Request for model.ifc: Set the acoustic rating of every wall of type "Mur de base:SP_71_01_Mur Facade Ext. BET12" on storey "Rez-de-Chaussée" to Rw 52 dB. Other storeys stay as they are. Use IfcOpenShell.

First a look at what the model holds.

```python
import ifcopenshell
import ifcopenshell.util.element

model = ifcopenshell.open("model.ifc")
print(model.schema)
storey = next(s for s in model.by_type("IfcBuildingStorey") if s.Name == "Rez-de-Chaussée")
walls = [e for e in ifcopenshell.util.element.get_decomposition(storey) if e.is_a("IfcWall")]
seen = {}
for e in walls:
    element_type = ifcopenshell.util.element.get_type(e)
    key = (element_type.Name if element_type != e and element_type else None, ifcopenshell.util.element.get_pset(e, "Pset_WallCommon", "AcousticRating"))
    seen[key] = seen.get(key, 0) + 1
for (name, value), count in sorted(seen.items(), key=str):
    print(count, "x", name, "|", value)
```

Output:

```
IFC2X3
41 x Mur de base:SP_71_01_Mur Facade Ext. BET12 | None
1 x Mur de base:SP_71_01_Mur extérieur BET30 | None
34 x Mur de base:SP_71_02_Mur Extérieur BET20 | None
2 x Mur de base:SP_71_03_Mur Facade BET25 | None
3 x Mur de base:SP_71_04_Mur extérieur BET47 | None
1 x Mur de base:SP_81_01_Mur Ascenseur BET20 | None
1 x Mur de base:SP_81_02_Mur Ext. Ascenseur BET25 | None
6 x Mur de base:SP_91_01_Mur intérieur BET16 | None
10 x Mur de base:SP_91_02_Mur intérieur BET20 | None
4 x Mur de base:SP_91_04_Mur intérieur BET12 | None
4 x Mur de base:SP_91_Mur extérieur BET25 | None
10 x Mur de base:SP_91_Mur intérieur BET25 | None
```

```python
import ifcopenshell
import ifcopenshell.api.pset
import ifcopenshell.util.element

model = ifcopenshell.open("model.ifc")

storey = next(s for s in model.by_type("IfcBuildingStorey") if s.Name == "Rez-de-Chaussée")
walls = [e for e in ifcopenshell.util.element.get_decomposition(storey) if e.is_a("IfcWall")]

count = 0
for e in walls:
    element_type = ifcopenshell.util.element.get_type(e)
    if element_type in (None, e) or element_type.Name != "Mur de base:SP_71_01_Mur Facade Ext. BET12":
        continue
    found = ifcopenshell.util.element.get_pset(e, "Pset_WallCommon", should_inherit=False)
    if found:
        pset = model.by_id(found["id"])
        if len(ifcopenshell.util.element.get_elements_by_pset(pset)) > 1:
            pset = ifcopenshell.api.pset.unshare_pset(model, products=[e], pset=pset)[0]
    else:
        pset = ifcopenshell.api.pset.add_pset(model, product=e, name="Pset_WallCommon")
    ifcopenshell.api.pset.edit_pset(model, pset=pset, properties={"AcousticRating": "Rw 52 dB"})
    count += 1

print(count, "walls updated")

model.write("model_updated.ifc")
```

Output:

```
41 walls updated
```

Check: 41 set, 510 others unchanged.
